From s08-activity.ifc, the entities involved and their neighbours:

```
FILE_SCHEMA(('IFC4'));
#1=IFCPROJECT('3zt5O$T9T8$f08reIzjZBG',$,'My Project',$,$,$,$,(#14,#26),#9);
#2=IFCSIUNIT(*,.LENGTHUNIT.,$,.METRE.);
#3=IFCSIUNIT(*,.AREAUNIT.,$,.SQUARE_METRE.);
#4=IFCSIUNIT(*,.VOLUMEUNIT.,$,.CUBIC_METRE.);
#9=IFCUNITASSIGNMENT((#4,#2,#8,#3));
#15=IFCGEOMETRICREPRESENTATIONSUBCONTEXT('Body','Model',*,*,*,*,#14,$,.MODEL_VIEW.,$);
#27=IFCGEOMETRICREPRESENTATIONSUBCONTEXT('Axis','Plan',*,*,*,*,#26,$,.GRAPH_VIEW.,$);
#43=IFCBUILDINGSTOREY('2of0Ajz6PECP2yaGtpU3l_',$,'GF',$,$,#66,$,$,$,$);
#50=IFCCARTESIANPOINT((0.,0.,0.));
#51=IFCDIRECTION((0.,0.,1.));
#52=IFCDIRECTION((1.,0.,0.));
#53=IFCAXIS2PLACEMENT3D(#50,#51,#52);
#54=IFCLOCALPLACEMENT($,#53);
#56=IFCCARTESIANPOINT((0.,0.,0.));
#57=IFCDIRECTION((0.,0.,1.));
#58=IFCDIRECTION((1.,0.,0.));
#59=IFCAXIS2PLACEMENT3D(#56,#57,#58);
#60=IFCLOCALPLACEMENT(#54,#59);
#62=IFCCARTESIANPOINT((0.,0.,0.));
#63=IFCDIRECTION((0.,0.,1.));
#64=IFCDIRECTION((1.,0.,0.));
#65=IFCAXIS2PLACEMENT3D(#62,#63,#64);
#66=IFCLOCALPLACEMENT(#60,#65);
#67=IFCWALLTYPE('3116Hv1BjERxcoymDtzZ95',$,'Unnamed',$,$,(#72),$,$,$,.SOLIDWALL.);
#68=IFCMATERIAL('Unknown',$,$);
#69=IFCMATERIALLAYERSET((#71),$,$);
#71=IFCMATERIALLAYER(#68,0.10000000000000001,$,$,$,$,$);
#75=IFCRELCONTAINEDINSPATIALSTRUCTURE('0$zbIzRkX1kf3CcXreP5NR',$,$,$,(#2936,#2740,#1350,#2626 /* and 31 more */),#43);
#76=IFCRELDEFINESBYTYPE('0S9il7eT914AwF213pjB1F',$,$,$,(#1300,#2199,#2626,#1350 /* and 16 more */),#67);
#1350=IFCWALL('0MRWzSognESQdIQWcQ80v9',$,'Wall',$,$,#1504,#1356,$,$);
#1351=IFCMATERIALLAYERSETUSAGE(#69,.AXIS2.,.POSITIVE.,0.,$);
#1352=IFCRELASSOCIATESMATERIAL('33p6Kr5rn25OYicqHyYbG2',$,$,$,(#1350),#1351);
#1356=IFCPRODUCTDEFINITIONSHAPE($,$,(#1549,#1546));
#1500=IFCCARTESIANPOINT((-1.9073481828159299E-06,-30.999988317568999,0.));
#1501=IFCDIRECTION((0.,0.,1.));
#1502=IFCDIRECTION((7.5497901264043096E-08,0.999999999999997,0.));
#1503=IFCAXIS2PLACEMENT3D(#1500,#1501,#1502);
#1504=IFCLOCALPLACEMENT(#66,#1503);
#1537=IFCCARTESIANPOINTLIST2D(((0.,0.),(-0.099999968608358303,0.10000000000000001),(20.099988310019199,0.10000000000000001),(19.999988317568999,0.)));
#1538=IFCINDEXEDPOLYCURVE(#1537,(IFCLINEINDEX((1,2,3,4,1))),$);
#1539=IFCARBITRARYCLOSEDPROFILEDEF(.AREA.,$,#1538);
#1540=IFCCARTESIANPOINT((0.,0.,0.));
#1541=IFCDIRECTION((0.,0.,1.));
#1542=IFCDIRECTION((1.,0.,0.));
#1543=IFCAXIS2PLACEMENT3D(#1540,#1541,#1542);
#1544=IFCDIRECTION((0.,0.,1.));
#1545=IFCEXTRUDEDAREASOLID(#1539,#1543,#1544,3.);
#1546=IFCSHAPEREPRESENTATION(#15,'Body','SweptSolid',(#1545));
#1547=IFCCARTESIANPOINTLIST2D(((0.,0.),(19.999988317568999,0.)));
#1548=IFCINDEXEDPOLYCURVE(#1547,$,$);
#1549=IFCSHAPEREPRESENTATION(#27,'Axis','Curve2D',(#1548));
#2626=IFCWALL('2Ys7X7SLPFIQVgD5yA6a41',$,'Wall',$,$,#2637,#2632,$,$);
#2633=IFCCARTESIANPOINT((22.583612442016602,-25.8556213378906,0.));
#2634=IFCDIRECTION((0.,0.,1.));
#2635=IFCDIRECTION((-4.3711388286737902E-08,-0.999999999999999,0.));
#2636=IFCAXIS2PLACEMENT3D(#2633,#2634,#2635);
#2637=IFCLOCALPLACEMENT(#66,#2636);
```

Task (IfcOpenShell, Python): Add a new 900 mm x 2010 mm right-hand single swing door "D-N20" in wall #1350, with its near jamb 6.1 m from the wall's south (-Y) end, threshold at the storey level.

```python
import numpy as np
import ifcopenshell
import ifcopenshell.api.feature
import ifcopenshell.api.geometry
import ifcopenshell.api.root
import ifcopenshell.api.spatial
import ifcopenshell.geom
import ifcopenshell.util.element
import ifcopenshell.util.placement
import ifcopenshell.util.representation
import ifcopenshell.util.shape
import ifcopenshell.util.unit

model = ifcopenshell.open("s08-activity.ifc")
unit_scale = ifcopenshell.util.unit.calculate_unit_scale(model)
settings = ifcopenshell.geom.settings()


def volume(element):
    """Net volume in cubic metres, openings subtracted."""
    shape = ifcopenshell.geom.create_shape(settings, element)
    return ifcopenshell.util.shape.get_volume(shape.geometry)


wall = model.by_guid("0MRWzSognESQdIQWcQ80v9")
storey = ifcopenshell.util.element.get_container(wall, ifc_class="IfcBuildingStorey")
context = ifcopenshell.util.representation.get_context(model, "Model", "Body", "MODEL_VIEW")
before = volume(wall)

width, height, from_end, sill = 0.9, 2.01, 6.1, 0.0  # metres

# The wall runs along its own X axis, and the end named is its -X end.
wall_shape = ifcopenshell.geom.create_shape(settings, wall)
x, y, z = ifcopenshell.util.shape.get_vertices(wall_shape.geometry).T
start = x.min() + from_end
face, thickness = float(y.min()), float(y.max() - y.min())
wall_matrix = ifcopenshell.util.placement.get_local_placement(wall.ObjectPlacement)
level = ifcopenshell.util.placement.get_local_placement(storey.ObjectPlacement)[2, 3]


def in_wall(x, y):
    """Placement at x, y metres in the wall's axes, at sill height."""
    matrix = wall_matrix.copy()
    matrix[:, 3] = wall_matrix @ np.array([x / unit_scale, y / unit_scale, 0.0, 1.0])
    matrix[2, 3] = level + sill / unit_scale
    return matrix


# Opening: a box that overshoots both wall faces by 50 mm.
opening = ifcopenshell.api.root.create_entity(model, ifc_class="IfcOpeningElement", predefined_type="OPENING")
box = ifcopenshell.api.geometry.add_wall_representation(
    model, context=context, length=width, height=height, thickness=thickness + 0.1
)
ifcopenshell.api.geometry.assign_representation(model, product=opening, representation=box)
ifcopenshell.api.geometry.edit_object_placement(model, product=opening, matrix=in_wall(start, face - 0.05), is_si=False)
ifcopenshell.api.feature.add_feature(model, feature=opening, element=wall)

door = ifcopenshell.api.root.create_entity(model, ifc_class="IfcDoor", name="D-N20", predefined_type="DOOR")
door.OverallWidth, door.OverallHeight = width / unit_scale, height / unit_scale
door.OperationType = "SINGLE_SWING_RIGHT"
body = ifcopenshell.api.geometry.add_door_representation(
    model,
    context=context,
    overall_width=door.OverallWidth,
    overall_height=door.OverallHeight,
    operation_type="SINGLE_SWING_RIGHT",
    lining_properties={"LiningDepth": thickness / unit_scale, "ThresholdDepth": thickness / unit_scale},
)
ifcopenshell.api.geometry.assign_representation(model, product=door, representation=body)
ifcopenshell.api.spatial.assign_container(model, products=[door], relating_structure=storey)
ifcopenshell.api.feature.add_filling(model, opening=opening, element=door)

# The lining spans the wall, so the door starts at the wall face.
ifcopenshell.api.geometry.edit_object_placement(model, product=door, matrix=in_wall(start, face), is_si=False)

after = volume(wall)

print(f"wall volume {before:.3f} -> {after:.3f} m3")

model.write("s08-activity_rev.ifc")
```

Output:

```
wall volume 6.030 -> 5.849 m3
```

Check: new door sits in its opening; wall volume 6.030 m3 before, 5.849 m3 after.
